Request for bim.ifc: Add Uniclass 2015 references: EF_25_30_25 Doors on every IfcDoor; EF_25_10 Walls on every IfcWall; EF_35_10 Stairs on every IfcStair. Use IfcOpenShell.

First a look at what the model holds.

```python
import ifcopenshell

model = ifcopenshell.open("bim.ifc")
print(model.schema)
print("classifications:", [c.Name for c in model.by_type("IfcClassification")])
for ifc_class in ("IfcDoor", "IfcRoof", "IfcStair", "IfcWall", "IfcWindow"):
    print(ifc_class, len(model.by_type(ifc_class)))
```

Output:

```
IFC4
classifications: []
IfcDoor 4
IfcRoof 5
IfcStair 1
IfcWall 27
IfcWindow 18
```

```python
import ifcopenshell
import ifcopenshell.api.classification

model = ifcopenshell.open("bim.ifc")

system = ifcopenshell.api.classification.add_classification(model, classification="Uniclass 2015")

codes = {
    "IfcDoor": ("EF_25_30_25", "Doors"),
    "IfcWall": ("EF_25_10", "Walls"),
    "IfcStair": ("EF_35_10", "Stairs"),
}
for ifc_class, (code, name) in codes.items():
    products = model.by_type(ifc_class)
    ifcopenshell.api.classification.add_reference(
        model, products=products, classification=system, identification=code, name=name
    )
    print(code, len(products))

model.write("bim_rev.ifc")
```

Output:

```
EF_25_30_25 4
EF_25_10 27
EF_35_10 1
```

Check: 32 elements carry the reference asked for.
